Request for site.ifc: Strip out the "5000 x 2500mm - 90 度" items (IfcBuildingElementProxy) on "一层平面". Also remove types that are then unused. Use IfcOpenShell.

First a look at what the model holds.

```python
import ifcopenshell
import ifcopenshell.util.element

model = ifcopenshell.open("site.ifc")
print(model.schema)
storey = next(s for s in model.by_type("IfcBuildingStorey") if s.Name == "一层平面")
proxies = [e for e in ifcopenshell.util.element.get_decomposition(storey) if e.is_a("IfcBuildingElementProxy")]
seen = {}
for e in proxies:
    element_type = ifcopenshell.util.element.get_type(e)
    name = element_type.Name if element_type not in (None, e) else None
    seen[name] = seen.get(name, 0) + 1
for name, count in sorted(seen.items(), key=str):
    print(count, "x", name)
```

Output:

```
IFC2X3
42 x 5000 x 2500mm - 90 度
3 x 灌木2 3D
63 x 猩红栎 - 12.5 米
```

```python
import ifcopenshell
import ifcopenshell.api.root
import ifcopenshell.util.element

model = ifcopenshell.open("site.ifc")

storey = next(s for s in model.by_type("IfcBuildingStorey") if s.Name == "一层平面")
proxies = [e for e in ifcopenshell.util.element.get_decomposition(storey) if e.is_a("IfcBuildingElementProxy")]
targets = [e for e in proxies if (t := ifcopenshell.util.element.get_type(e)) not in (None, e) and t.Name == "5000 x 2500mm - 90 度"]
types = {ifcopenshell.util.element.get_type(e) for e in targets} - {None, *targets}

for e in targets:
    ifcopenshell.api.root.remove_product(model, product=e)
print(len(targets), "removed")

unused = [t for t in types if not ifcopenshell.util.element.get_types(t)]
for t in unused:
    ifcopenshell.api.root.remove_product(model, product=t)
print(len(unused), "unused types removed")

model.write("site_v2.ifc")
```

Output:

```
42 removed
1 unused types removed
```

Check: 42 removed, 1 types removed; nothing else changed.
